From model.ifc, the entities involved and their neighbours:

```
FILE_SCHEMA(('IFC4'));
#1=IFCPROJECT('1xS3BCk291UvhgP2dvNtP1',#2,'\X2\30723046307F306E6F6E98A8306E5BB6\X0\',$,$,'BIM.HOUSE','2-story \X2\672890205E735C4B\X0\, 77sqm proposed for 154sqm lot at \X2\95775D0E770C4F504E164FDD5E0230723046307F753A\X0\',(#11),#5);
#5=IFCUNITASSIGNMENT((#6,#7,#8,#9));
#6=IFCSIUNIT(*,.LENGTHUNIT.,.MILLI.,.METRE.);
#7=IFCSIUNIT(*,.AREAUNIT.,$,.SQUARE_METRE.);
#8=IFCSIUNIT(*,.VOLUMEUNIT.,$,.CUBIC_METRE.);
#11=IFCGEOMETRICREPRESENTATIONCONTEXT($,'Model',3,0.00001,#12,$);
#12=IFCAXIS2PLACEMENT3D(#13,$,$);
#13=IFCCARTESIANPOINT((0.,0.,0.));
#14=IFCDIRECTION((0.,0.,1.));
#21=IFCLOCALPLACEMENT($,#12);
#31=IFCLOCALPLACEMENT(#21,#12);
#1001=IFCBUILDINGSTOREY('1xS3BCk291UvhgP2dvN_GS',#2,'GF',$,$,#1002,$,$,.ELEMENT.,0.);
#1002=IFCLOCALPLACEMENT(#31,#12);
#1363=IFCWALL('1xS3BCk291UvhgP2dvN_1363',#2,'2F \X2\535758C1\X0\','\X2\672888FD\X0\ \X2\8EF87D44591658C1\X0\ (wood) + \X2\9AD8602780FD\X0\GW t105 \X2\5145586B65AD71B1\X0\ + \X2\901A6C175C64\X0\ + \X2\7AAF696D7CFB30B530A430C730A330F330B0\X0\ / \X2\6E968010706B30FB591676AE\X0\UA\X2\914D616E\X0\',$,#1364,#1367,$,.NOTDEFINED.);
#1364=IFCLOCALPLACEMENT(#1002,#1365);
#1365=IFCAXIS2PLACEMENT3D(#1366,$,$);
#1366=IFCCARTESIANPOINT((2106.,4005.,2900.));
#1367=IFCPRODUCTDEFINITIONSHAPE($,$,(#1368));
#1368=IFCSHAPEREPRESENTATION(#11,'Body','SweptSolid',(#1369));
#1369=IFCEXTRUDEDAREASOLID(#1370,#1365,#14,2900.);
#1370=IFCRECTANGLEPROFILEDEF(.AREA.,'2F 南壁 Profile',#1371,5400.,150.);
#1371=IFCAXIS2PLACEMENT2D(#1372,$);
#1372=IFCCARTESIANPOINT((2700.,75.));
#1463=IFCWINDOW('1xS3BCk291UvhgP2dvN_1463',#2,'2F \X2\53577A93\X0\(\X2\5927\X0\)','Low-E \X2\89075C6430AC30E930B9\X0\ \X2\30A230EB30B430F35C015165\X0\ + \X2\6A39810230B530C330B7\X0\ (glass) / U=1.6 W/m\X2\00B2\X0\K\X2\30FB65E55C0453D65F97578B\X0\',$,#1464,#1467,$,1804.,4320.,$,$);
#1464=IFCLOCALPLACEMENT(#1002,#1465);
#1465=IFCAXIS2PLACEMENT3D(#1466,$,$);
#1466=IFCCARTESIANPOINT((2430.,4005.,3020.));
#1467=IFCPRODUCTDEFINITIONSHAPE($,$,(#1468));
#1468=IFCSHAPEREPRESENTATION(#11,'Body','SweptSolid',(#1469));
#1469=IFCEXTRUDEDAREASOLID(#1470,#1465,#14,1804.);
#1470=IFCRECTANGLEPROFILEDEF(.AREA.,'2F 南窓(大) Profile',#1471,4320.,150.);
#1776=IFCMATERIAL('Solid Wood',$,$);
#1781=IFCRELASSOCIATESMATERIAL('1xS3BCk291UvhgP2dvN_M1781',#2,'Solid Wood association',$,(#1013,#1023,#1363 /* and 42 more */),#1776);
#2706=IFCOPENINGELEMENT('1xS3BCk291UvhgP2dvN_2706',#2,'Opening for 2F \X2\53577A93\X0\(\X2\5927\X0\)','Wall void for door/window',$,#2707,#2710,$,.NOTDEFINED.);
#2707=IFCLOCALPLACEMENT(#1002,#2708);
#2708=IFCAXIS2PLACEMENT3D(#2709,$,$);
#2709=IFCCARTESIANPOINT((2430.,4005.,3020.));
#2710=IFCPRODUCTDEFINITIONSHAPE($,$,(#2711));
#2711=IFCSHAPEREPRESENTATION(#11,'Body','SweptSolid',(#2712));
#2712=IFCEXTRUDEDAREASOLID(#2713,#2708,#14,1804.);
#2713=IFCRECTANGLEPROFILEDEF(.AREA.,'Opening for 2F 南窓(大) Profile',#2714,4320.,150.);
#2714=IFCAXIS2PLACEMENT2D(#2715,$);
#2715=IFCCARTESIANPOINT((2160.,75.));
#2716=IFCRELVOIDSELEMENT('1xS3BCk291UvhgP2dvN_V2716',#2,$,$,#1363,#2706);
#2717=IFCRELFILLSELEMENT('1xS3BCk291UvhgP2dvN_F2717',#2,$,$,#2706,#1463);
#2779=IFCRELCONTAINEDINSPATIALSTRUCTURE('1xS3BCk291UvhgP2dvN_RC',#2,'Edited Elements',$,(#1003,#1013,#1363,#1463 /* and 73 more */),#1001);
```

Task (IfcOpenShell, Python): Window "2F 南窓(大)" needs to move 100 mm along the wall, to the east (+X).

```python
import ifcopenshell
import ifcopenshell.api.geometry
import ifcopenshell.util.placement
import ifcopenshell.util.unit

model = ifcopenshell.open("model.ifc")
unit_scale = ifcopenshell.util.unit.calculate_unit_scale(model)

window = model.by_guid("1xS3BCk291UvhgP2dvN_1463")
opening = window.FillsVoids[0].RelatingOpeningElement
wall = opening.VoidsElements[0].RelatingBuildingElement

wall_matrix = ifcopenshell.util.placement.get_local_placement(wall.ObjectPlacement)
shift = wall_matrix[:3, 0] * 0.1 / unit_scale
before = ifcopenshell.util.placement.get_local_placement(window.ObjectPlacement)[:3, 3].copy()

# The window is not placed relative to its opening, so move both.
for product in (opening, window):
    matrix = ifcopenshell.util.placement.get_local_placement(product.ObjectPlacement)
    matrix[:3, 3] += shift
    ifcopenshell.api.geometry.edit_object_placement(model, product=product, matrix=matrix, is_si=False)

after = ifcopenshell.util.placement.get_local_placement(window.ObjectPlacement)[:3, 3]
print("window moved by", (after - before).round(3) + 0.0)

model.write("model_updated.ifc")
```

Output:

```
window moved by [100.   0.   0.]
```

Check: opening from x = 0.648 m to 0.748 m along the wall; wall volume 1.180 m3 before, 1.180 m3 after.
